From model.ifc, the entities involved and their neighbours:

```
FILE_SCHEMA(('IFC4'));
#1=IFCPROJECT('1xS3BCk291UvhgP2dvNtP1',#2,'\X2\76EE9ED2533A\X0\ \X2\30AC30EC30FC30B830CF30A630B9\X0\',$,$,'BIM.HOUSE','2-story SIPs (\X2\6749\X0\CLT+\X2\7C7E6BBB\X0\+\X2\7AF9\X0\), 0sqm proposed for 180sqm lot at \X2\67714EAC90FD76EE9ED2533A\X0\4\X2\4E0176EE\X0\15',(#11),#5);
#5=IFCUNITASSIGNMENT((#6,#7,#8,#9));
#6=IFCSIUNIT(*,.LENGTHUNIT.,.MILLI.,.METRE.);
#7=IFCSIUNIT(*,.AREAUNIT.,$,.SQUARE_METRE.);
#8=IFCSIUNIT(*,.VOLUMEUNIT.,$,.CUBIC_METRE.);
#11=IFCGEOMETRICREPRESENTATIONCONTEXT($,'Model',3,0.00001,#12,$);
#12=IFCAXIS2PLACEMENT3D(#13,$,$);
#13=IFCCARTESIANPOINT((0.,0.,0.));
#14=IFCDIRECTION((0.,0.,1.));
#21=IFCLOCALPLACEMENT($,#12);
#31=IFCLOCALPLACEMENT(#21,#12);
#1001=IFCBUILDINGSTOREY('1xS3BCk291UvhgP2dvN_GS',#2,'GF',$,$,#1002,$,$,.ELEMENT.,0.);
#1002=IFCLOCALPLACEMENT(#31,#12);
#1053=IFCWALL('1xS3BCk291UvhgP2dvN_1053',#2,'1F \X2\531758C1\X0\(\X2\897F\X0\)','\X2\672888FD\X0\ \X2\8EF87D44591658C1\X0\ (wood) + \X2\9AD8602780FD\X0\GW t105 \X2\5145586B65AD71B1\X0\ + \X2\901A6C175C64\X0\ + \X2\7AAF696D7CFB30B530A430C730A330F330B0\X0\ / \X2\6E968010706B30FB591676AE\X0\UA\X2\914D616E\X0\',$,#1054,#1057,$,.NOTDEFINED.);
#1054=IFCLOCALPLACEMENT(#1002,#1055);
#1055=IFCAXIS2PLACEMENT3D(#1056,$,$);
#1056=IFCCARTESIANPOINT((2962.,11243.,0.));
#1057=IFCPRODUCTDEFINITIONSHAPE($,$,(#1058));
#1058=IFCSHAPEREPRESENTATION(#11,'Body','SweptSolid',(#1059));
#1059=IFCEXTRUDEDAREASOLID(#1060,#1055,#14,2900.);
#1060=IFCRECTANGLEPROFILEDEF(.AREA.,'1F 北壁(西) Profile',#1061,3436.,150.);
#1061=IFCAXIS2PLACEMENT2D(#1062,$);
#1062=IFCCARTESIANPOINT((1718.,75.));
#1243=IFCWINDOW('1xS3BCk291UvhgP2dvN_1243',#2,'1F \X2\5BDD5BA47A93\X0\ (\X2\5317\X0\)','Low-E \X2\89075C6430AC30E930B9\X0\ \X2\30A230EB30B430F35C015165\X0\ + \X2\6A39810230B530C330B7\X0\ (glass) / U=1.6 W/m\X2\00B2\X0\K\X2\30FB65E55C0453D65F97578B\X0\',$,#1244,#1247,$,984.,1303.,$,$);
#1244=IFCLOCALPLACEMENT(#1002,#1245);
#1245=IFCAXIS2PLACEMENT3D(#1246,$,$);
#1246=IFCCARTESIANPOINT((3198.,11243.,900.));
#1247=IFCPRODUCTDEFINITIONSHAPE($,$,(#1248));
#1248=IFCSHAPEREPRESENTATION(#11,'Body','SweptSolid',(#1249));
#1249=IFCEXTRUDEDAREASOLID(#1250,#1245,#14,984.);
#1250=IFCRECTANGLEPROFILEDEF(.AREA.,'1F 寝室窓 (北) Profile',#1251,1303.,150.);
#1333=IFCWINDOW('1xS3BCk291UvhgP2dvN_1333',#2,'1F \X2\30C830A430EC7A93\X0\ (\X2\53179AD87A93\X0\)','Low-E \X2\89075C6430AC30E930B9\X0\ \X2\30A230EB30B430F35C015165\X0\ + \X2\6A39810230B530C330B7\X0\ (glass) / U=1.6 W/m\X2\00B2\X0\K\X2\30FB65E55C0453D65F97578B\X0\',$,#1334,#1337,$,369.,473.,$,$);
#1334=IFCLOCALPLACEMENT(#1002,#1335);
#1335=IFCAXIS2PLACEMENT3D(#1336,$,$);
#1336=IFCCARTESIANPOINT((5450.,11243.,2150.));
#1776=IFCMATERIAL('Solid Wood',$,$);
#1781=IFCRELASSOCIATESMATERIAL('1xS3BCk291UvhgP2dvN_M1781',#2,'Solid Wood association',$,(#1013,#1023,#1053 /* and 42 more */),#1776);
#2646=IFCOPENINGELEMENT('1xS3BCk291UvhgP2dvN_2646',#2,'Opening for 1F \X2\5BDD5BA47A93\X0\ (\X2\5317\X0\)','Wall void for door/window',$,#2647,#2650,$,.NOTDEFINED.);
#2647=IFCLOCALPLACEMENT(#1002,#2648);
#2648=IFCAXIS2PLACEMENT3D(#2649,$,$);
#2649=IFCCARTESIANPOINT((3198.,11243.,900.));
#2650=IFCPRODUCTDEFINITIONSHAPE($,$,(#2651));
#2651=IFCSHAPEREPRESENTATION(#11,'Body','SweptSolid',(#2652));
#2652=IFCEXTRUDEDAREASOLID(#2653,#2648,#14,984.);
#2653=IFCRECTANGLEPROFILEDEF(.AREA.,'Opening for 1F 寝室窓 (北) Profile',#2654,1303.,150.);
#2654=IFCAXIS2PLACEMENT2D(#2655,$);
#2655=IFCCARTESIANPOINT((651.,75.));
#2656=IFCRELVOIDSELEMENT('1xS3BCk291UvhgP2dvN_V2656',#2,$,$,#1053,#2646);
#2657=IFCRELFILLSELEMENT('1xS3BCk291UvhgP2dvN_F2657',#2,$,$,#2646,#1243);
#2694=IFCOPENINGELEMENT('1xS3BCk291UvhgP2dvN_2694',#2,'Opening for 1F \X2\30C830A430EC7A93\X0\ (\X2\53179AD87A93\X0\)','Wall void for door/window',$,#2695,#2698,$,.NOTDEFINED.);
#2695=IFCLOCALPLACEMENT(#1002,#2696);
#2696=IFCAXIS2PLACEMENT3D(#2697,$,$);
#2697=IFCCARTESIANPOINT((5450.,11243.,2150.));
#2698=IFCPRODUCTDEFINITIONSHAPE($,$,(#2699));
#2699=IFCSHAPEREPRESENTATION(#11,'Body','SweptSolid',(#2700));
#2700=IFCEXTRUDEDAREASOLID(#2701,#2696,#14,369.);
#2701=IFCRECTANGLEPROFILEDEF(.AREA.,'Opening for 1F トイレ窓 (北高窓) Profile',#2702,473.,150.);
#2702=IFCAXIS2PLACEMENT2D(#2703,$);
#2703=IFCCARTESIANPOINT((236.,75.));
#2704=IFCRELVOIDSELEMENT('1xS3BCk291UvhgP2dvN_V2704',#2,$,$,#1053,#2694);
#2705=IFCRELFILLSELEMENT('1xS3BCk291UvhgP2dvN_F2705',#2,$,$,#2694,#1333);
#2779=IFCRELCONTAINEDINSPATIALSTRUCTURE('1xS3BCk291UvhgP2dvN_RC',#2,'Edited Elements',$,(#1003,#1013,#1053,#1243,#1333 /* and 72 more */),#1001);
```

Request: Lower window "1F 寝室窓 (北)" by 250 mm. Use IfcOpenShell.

```python
import numpy as np
import ifcopenshell
import ifcopenshell.api.geometry
import ifcopenshell.util.placement
import ifcopenshell.util.unit

model = ifcopenshell.open("model.ifc")
unit_scale = ifcopenshell.util.unit.calculate_unit_scale(model)

window = model.by_guid("1xS3BCk291UvhgP2dvN_1243")
opening = window.FillsVoids[0].RelatingOpeningElement
dz = -250.0

shift = np.array([0.0, 0.0, dz])
# The window is not placed relative to its opening, so move both.
for product in (opening, window):
    matrix = ifcopenshell.util.placement.get_local_placement(product.ObjectPlacement)
    matrix[:3, 3] += shift
    ifcopenshell.api.geometry.edit_object_placement(model, product=product, matrix=matrix, is_si=False)

print(f"moved by {dz * unit_scale:+.3f} m")

model.write("model-out.ifc")
```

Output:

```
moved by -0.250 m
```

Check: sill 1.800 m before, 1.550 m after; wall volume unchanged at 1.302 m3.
